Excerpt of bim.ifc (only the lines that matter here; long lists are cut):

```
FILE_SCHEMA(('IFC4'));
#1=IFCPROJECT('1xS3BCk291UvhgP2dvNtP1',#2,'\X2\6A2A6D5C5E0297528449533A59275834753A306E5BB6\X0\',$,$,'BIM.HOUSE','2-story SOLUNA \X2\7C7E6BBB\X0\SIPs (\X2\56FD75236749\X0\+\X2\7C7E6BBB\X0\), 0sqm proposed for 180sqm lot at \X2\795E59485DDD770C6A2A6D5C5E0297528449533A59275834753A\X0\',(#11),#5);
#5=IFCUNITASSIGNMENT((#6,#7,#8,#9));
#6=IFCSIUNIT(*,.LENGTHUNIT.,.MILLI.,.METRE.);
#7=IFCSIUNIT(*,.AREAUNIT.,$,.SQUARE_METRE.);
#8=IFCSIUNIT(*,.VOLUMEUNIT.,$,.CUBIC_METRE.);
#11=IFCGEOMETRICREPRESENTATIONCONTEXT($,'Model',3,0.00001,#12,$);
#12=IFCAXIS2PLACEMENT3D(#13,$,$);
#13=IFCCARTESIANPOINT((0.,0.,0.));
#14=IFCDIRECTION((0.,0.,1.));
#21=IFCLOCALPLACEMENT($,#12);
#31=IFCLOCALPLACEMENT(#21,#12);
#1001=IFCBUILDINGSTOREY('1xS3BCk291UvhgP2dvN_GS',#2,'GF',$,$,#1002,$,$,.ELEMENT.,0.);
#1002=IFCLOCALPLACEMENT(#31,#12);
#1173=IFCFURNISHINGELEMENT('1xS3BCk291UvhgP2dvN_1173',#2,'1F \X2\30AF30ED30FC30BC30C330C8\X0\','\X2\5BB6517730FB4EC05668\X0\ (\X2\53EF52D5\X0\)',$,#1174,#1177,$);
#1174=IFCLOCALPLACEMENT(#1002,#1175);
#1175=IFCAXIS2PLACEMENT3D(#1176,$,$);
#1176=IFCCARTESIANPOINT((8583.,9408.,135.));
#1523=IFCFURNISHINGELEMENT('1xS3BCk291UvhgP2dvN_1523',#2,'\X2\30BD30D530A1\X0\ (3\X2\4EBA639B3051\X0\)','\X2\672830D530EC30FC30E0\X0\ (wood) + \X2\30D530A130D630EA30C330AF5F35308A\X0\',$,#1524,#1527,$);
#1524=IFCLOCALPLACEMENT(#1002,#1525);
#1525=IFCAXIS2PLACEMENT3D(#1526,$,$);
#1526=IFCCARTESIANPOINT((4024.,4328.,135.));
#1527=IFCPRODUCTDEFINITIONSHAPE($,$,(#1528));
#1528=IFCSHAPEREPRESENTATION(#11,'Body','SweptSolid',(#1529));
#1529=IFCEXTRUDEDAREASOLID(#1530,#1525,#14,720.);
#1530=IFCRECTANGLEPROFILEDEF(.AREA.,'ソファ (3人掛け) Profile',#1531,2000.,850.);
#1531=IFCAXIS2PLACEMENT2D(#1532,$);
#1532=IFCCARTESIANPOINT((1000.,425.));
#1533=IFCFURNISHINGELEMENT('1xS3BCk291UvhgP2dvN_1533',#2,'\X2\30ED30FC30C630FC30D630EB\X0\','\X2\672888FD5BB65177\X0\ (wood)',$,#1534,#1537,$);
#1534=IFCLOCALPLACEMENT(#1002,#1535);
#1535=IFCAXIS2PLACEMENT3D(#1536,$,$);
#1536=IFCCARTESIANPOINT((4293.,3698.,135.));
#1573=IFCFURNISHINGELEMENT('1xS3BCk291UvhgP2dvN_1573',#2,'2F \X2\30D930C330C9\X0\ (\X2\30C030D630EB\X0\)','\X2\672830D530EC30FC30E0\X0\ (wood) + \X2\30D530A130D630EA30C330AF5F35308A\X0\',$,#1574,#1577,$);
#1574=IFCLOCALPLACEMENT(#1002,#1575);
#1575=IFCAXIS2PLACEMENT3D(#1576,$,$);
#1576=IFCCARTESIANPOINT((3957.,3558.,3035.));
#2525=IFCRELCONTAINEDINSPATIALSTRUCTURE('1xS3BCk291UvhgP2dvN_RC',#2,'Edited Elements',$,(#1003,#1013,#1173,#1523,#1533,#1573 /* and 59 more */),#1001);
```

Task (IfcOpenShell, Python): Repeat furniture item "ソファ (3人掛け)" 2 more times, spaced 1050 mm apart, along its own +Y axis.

```python
import ifcopenshell
import ifcopenshell.api.geometry
import ifcopenshell.api.root
import ifcopenshell.util.element
import ifcopenshell.util.placement

model = ifcopenshell.open("bim.ifc")


def reuse_history(source, copy):
    """copy_class also copies each property set's owner history, people and application; keep the originals."""
    for rel in copy.IsDefinedBy:
        if rel.is_a("IfcRelDefinesByProperties") and (history := rel.RelatingPropertyDefinition.OwnerHistory):
            rel.RelatingPropertyDefinition.OwnerHistory = source.OwnerHistory
            ifcopenshell.util.element.remove_deep2(model, history)


source = model.by_guid("1xS3BCk291UvhgP2dvN_1523")
base = ifcopenshell.util.placement.get_local_placement(source.ObjectPlacement)
step = base[:3, 1] * 1050.0

for i in range(1, 3):
    copy = ifcopenshell.api.root.copy_class(model, product=source)
    copy.Representation = ifcopenshell.util.element.copy_deep(
        model, source.Representation, exclude=["IfcGeometricRepresentationContext", "IfcRepresentationMap"]
    )
    reuse_history(source, copy)
    matrix = base.copy()
    matrix[:3, 3] += i * step
    print("added at", matrix[:3, 3].round(3) + 0.0)
    ifcopenshell.api.geometry.edit_object_placement(model, product=copy, matrix=matrix, is_si=False)

model.write("bim_edited.ifc")
```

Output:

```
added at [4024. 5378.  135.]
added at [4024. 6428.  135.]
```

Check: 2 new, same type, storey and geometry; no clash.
